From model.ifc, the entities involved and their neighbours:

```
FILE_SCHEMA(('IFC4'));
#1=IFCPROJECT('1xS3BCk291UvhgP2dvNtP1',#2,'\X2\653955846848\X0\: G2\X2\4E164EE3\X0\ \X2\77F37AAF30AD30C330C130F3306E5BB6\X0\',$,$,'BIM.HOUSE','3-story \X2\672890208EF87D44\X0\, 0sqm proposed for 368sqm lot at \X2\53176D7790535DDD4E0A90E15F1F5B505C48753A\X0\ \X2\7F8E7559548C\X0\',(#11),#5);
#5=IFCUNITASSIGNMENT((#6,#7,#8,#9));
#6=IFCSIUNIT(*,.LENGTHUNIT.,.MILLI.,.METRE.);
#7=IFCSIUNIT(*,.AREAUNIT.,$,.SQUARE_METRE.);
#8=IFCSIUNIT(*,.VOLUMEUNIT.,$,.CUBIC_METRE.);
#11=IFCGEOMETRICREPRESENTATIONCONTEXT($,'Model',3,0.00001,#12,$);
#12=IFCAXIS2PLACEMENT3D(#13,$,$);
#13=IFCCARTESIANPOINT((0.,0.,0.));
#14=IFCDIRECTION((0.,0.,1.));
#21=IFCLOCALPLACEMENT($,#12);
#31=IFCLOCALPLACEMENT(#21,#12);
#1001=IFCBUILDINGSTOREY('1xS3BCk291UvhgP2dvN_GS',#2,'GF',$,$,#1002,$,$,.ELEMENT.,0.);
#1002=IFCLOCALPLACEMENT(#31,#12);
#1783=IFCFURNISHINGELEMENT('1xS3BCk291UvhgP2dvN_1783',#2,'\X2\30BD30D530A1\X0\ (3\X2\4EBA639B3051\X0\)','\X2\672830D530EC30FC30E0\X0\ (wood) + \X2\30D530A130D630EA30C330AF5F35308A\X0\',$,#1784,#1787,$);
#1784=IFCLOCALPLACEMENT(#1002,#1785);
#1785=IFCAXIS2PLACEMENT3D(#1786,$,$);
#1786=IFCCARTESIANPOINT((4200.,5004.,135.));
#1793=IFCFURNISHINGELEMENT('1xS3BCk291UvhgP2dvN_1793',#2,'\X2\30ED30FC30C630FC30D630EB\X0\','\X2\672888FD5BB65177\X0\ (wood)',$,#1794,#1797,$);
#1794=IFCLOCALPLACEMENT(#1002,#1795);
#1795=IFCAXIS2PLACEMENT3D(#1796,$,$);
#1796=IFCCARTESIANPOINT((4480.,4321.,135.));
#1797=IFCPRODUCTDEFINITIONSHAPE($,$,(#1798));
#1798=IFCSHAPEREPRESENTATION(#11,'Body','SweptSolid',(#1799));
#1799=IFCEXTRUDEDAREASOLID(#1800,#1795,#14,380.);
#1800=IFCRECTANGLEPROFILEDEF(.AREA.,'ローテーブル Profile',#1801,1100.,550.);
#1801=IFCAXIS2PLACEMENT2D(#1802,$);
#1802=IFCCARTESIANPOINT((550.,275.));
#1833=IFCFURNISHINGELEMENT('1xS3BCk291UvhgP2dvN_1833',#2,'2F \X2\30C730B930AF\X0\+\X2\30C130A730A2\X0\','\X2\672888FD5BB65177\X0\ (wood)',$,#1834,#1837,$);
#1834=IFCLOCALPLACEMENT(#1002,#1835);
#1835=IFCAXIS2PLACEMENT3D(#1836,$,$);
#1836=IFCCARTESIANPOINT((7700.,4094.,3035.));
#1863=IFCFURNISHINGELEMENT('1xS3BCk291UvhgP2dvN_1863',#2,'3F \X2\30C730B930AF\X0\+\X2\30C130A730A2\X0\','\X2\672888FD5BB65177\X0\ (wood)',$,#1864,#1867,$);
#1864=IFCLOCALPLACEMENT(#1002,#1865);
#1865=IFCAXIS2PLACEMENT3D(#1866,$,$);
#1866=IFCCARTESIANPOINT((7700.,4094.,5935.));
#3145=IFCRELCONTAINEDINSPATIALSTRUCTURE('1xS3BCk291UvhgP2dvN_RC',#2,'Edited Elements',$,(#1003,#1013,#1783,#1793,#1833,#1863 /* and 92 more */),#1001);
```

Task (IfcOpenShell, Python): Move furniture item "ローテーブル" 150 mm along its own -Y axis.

```python
import ifcopenshell
import ifcopenshell.api.geometry
import ifcopenshell.util.placement
import ifcopenshell.util.unit

model = ifcopenshell.open("model.ifc")
unit_scale = ifcopenshell.util.unit.calculate_unit_scale(model)

item = model.by_guid("1xS3BCk291UvhgP2dvN_1793")
matrix = ifcopenshell.util.placement.get_local_placement(item.ObjectPlacement)
matrix[:3, 3] -= matrix[:3, 1] * 0.15 / unit_scale
ifcopenshell.api.geometry.edit_object_placement(model, product=item, matrix=matrix, is_si=False)

print(ifcopenshell.util.placement.get_local_placement(item.ObjectPlacement).round(3) + 0.0)

model.write("model_edited.ifc")
```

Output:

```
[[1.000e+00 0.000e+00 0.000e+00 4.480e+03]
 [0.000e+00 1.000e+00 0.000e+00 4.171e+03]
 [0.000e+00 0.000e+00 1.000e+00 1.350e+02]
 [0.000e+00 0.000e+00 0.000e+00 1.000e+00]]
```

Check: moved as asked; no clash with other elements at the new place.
